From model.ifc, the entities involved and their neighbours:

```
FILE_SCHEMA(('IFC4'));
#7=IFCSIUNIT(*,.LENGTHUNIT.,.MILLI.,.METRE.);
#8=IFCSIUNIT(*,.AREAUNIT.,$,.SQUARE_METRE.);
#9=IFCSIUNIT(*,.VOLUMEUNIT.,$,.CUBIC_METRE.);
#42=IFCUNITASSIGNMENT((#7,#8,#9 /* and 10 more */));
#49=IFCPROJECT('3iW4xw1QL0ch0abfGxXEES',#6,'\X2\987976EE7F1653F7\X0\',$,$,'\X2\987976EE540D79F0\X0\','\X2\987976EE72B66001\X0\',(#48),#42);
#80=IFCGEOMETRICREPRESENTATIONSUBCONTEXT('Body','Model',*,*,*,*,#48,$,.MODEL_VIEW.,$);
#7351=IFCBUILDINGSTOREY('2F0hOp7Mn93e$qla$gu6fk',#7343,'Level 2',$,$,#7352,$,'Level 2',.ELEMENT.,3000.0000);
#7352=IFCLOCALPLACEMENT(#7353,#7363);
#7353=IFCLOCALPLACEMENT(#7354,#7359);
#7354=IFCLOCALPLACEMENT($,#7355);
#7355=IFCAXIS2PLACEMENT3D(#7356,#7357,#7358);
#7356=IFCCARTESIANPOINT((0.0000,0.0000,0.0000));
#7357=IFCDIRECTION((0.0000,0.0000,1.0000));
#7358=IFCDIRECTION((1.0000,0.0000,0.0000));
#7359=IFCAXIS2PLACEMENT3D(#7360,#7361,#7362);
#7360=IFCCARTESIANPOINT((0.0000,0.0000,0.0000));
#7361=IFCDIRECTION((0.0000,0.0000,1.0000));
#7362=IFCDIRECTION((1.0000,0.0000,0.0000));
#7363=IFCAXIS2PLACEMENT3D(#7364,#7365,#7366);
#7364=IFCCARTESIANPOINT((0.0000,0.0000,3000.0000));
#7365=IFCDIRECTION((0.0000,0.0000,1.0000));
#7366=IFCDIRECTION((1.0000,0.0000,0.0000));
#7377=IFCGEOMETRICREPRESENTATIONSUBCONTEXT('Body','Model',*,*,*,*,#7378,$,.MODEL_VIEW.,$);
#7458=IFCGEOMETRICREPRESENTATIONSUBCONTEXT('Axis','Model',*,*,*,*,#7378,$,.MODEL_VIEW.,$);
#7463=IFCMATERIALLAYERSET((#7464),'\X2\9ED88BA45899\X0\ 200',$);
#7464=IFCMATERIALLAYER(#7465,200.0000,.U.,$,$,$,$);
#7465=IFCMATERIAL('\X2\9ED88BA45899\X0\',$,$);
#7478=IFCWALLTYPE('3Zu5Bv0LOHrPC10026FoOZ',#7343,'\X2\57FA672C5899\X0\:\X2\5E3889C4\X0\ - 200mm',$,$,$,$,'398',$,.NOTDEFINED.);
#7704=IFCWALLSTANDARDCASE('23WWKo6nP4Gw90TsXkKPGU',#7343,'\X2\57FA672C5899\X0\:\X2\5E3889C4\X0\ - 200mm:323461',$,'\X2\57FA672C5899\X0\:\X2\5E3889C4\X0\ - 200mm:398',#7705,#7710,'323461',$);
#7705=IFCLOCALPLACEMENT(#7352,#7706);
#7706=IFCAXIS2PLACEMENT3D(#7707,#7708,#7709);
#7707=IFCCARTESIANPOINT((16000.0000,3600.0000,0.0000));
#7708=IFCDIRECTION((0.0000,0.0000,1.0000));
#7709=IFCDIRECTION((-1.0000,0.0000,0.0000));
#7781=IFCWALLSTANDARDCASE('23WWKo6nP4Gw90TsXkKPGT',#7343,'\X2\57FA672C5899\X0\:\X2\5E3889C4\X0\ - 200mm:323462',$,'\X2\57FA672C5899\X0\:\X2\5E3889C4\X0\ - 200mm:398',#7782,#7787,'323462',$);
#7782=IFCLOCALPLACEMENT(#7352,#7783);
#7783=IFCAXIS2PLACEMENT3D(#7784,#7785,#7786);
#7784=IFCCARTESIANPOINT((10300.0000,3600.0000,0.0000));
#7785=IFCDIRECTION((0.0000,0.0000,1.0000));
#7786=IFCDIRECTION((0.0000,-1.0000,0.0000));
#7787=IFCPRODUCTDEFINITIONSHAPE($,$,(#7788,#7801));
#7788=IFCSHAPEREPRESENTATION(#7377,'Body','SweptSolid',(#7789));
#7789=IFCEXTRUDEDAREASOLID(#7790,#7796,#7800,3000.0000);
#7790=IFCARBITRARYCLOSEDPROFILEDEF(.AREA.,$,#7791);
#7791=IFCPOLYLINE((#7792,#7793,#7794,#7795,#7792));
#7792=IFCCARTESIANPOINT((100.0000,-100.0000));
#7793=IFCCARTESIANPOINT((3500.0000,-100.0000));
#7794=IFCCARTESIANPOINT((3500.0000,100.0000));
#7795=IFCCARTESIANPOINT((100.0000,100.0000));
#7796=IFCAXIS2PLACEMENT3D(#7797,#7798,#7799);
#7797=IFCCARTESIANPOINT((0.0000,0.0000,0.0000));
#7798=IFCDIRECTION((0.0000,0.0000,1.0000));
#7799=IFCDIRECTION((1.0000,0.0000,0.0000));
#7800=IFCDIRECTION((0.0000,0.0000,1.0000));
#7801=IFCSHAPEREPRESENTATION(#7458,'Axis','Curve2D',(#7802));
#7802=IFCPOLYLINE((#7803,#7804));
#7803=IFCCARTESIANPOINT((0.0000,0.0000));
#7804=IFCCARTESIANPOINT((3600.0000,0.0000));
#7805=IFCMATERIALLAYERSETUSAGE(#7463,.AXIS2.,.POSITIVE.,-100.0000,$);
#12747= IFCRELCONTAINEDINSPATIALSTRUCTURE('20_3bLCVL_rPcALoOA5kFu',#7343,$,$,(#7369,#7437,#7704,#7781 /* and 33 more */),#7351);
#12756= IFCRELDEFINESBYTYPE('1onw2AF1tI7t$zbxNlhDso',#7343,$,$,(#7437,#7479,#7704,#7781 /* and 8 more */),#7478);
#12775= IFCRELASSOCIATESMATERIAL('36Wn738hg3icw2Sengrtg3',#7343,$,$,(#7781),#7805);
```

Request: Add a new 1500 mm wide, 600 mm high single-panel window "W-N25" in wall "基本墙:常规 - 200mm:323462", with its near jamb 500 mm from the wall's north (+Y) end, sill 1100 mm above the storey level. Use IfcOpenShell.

```python
import numpy as np
import ifcopenshell
import ifcopenshell.api.feature
import ifcopenshell.api.geometry
import ifcopenshell.api.root
import ifcopenshell.api.spatial
import ifcopenshell.geom
import ifcopenshell.util.element
import ifcopenshell.util.placement
import ifcopenshell.util.representation
import ifcopenshell.util.shape
import ifcopenshell.util.unit

model = ifcopenshell.open("model.ifc")
unit_scale = ifcopenshell.util.unit.calculate_unit_scale(model)
settings = ifcopenshell.geom.settings()


def volume(element):
    """Net volume in cubic metres, openings subtracted."""
    shape = ifcopenshell.geom.create_shape(settings, element)
    return ifcopenshell.util.shape.get_volume(shape.geometry)


wall = model.by_guid("23WWKo6nP4Gw90TsXkKPGT")
storey = ifcopenshell.util.element.get_container(wall, ifc_class="IfcBuildingStorey")
context = ifcopenshell.util.representation.get_context(model, "Model", "Body", "MODEL_VIEW")
before = volume(wall)

width, height, from_end, sill = 1.5, 0.6, 0.5, 1.1  # metres

# The wall runs along its own X axis, and the end named is its -X end.
wall_shape = ifcopenshell.geom.create_shape(settings, wall)
x, y, z = ifcopenshell.util.shape.get_vertices(wall_shape.geometry).T
start = x.min() + from_end
face, thickness = float(y.min()), float(y.max() - y.min())
wall_matrix = ifcopenshell.util.placement.get_local_placement(wall.ObjectPlacement)
level = ifcopenshell.util.placement.get_local_placement(storey.ObjectPlacement)[2, 3]


def in_wall(x, y):
    """Placement at x, y metres in the wall's axes, at sill height."""
    matrix = wall_matrix.copy()
    matrix[:, 3] = wall_matrix @ np.array([x / unit_scale, y / unit_scale, 0.0, 1.0])
    matrix[2, 3] = level + sill / unit_scale
    return matrix


# Opening: a box that overshoots both wall faces by 50 mm.
opening = ifcopenshell.api.root.create_entity(model, ifc_class="IfcOpeningElement", predefined_type="OPENING")
box = ifcopenshell.api.geometry.add_wall_representation(
    model, context=context, length=width, height=height, thickness=thickness + 0.1
)
ifcopenshell.api.geometry.assign_representation(model, product=opening, representation=box)
ifcopenshell.api.geometry.edit_object_placement(model, product=opening, matrix=in_wall(start, face - 0.05), is_si=False)
ifcopenshell.api.feature.add_feature(model, feature=opening, element=wall)

window = ifcopenshell.api.root.create_entity(model, ifc_class="IfcWindow", name="W-N25", predefined_type="WINDOW")
window.OverallWidth, window.OverallHeight = width / unit_scale, height / unit_scale
window.PartitioningType = "SINGLE_PANEL"
body = ifcopenshell.api.geometry.add_window_representation(
    model,
    context=context,
    overall_width=window.OverallWidth,
    overall_height=window.OverallHeight,
    partition_type="SINGLE_PANEL",
)
ifcopenshell.api.geometry.assign_representation(model, product=window, representation=body)
ifcopenshell.api.spatial.assign_container(model, products=[window], relating_structure=storey)
ifcopenshell.api.feature.add_filling(model, opening=opening, element=window)

# Centre the window in the wall's thickness.
ifcopenshell.api.geometry.edit_object_placement(model, product=window, matrix=in_wall(start, face), is_si=False)
window_shape = ifcopenshell.geom.create_shape(settings, window)
depth = ifcopenshell.util.shape.get_vertices(window_shape.geometry)[:, 1]
offset = face + thickness / 2 - (depth.min() + depth.max()) / 2
ifcopenshell.api.geometry.edit_object_placement(model, product=window, matrix=in_wall(start, offset), is_si=False)

after = volume(wall)

print(f"wall volume {before:.3f} -> {after:.3f} m3")

model.write("model_edited.ifc")
```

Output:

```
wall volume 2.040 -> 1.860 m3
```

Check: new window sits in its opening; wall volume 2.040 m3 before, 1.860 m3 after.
